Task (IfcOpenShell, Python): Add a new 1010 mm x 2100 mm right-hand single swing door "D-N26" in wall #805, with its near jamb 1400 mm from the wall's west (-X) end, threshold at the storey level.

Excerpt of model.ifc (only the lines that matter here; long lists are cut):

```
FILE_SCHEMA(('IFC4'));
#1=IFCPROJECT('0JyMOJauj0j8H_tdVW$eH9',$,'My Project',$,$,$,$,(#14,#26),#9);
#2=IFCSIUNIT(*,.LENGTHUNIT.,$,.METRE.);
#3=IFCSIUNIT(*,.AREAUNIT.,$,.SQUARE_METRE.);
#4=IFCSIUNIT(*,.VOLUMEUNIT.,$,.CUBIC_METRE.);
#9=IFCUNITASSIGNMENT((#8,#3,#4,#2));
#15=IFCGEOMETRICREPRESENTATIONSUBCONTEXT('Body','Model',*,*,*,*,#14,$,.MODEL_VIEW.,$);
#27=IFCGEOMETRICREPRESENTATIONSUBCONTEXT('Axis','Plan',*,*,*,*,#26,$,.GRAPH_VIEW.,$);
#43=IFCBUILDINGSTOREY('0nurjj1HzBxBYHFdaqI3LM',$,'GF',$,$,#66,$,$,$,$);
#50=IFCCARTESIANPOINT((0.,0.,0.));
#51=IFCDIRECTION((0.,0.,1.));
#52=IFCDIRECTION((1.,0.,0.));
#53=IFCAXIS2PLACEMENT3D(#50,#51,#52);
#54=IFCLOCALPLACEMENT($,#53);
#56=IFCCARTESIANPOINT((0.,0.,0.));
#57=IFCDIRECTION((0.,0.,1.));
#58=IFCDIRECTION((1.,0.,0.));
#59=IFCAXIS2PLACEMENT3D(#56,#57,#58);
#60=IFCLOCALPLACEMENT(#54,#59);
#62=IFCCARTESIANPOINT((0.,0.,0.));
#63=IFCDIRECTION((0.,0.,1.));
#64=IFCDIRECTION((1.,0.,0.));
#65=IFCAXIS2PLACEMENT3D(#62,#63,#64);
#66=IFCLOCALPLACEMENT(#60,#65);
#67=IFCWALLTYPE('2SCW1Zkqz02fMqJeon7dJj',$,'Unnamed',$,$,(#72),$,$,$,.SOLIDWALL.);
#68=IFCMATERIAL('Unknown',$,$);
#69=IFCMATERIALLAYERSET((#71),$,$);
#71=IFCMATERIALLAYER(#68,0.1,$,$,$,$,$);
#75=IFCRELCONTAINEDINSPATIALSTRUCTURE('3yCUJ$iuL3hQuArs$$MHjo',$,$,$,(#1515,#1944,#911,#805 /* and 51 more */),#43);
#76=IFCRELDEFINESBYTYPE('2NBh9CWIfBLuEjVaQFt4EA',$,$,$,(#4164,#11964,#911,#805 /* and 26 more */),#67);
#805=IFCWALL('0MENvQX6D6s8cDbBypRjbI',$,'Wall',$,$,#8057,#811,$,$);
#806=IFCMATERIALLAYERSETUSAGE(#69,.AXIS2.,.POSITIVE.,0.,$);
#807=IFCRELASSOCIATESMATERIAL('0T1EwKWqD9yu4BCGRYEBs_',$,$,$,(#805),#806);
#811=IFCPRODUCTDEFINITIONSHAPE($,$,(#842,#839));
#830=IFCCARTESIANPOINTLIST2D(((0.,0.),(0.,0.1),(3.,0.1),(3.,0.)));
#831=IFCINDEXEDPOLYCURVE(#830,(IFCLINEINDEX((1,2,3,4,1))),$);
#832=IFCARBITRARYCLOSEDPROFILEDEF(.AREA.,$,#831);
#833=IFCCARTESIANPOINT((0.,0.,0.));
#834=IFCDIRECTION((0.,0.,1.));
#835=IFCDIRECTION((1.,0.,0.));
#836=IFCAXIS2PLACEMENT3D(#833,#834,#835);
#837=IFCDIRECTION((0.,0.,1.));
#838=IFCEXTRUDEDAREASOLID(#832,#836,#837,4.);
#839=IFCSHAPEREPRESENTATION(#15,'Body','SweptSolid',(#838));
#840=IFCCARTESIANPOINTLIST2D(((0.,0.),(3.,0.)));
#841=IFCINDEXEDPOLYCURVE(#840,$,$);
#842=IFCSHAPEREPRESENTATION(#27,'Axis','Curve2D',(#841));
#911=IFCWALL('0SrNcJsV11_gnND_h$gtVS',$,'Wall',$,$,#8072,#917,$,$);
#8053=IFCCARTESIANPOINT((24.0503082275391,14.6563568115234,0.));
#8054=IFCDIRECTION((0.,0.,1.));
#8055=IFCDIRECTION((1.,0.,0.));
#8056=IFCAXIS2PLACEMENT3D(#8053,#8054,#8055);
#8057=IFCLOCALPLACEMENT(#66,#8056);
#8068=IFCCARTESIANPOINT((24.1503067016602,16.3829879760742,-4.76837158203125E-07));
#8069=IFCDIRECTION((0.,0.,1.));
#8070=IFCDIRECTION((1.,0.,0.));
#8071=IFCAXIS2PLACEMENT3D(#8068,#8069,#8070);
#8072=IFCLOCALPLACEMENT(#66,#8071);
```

```python
import numpy as np
import ifcopenshell
import ifcopenshell.api.feature
import ifcopenshell.api.geometry
import ifcopenshell.api.root
import ifcopenshell.api.spatial
import ifcopenshell.geom
import ifcopenshell.util.element
import ifcopenshell.util.placement
import ifcopenshell.util.representation
import ifcopenshell.util.shape
import ifcopenshell.util.unit

model = ifcopenshell.open("model.ifc")
unit_scale = ifcopenshell.util.unit.calculate_unit_scale(model)
settings = ifcopenshell.geom.settings()


def volume(element):
    """Net volume in cubic metres, openings subtracted."""
    shape = ifcopenshell.geom.create_shape(settings, element)
    return ifcopenshell.util.shape.get_volume(shape.geometry)


wall = model.by_id(805)
storey = ifcopenshell.util.element.get_container(wall, ifc_class="IfcBuildingStorey")
context = ifcopenshell.util.representation.get_context(model, "Model", "Body", "MODEL_VIEW")
before = volume(wall)

width, height, from_end, sill = 1.01, 2.1, 1.4, 0.0  # metres

# The wall runs along its own X axis, and the end named is its -X end.
wall_shape = ifcopenshell.geom.create_shape(settings, wall)
x, y, z = ifcopenshell.util.shape.get_vertices(wall_shape.geometry).T
start = x.min() + from_end
face, thickness = float(y.min()), float(y.max() - y.min())
wall_matrix = ifcopenshell.util.placement.get_local_placement(wall.ObjectPlacement)
level = ifcopenshell.util.placement.get_local_placement(storey.ObjectPlacement)[2, 3]


def in_wall(x, y):
    """Placement at x, y metres in the wall's axes, at sill height."""
    matrix = wall_matrix.copy()
    matrix[:, 3] = wall_matrix @ np.array([x / unit_scale, y / unit_scale, 0.0, 1.0])
    matrix[2, 3] = level + sill / unit_scale
    return matrix


# Opening: a box that overshoots both wall faces by 50 mm.
opening = ifcopenshell.api.root.create_entity(model, ifc_class="IfcOpeningElement", predefined_type="OPENING")
box = ifcopenshell.api.geometry.add_wall_representation(
    model, context=context, length=width, height=height, thickness=thickness + 0.1
)
ifcopenshell.api.geometry.assign_representation(model, product=opening, representation=box)
ifcopenshell.api.geometry.edit_object_placement(model, product=opening, matrix=in_wall(start, face - 0.05), is_si=False)
ifcopenshell.api.feature.add_feature(model, feature=opening, element=wall)

door = ifcopenshell.api.root.create_entity(model, ifc_class="IfcDoor", name="D-N26", predefined_type="DOOR")
door.OverallWidth, door.OverallHeight = width / unit_scale, height / unit_scale
door.OperationType = "SINGLE_SWING_RIGHT"
body = ifcopenshell.api.geometry.add_door_representation(
    model,
    context=context,
    overall_width=door.OverallWidth,
    overall_height=door.OverallHeight,
    operation_type="SINGLE_SWING_RIGHT",
    lining_properties={"LiningDepth": thickness / unit_scale, "ThresholdDepth": thickness / unit_scale},
)
ifcopenshell.api.geometry.assign_representation(model, product=door, representation=body)
ifcopenshell.api.spatial.assign_container(model, products=[door], relating_structure=storey)
ifcopenshell.api.feature.add_filling(model, opening=opening, element=door)

# The lining spans the wall, so the door starts at the wall face.
ifcopenshell.api.geometry.edit_object_placement(model, product=door, matrix=in_wall(start, face), is_si=False)

after = volume(wall)

print(f"wall volume {before:.3f} -> {after:.3f} m3")

model.write("model-out.ifc")
```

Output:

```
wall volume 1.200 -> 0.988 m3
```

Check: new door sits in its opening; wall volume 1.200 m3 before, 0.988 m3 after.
